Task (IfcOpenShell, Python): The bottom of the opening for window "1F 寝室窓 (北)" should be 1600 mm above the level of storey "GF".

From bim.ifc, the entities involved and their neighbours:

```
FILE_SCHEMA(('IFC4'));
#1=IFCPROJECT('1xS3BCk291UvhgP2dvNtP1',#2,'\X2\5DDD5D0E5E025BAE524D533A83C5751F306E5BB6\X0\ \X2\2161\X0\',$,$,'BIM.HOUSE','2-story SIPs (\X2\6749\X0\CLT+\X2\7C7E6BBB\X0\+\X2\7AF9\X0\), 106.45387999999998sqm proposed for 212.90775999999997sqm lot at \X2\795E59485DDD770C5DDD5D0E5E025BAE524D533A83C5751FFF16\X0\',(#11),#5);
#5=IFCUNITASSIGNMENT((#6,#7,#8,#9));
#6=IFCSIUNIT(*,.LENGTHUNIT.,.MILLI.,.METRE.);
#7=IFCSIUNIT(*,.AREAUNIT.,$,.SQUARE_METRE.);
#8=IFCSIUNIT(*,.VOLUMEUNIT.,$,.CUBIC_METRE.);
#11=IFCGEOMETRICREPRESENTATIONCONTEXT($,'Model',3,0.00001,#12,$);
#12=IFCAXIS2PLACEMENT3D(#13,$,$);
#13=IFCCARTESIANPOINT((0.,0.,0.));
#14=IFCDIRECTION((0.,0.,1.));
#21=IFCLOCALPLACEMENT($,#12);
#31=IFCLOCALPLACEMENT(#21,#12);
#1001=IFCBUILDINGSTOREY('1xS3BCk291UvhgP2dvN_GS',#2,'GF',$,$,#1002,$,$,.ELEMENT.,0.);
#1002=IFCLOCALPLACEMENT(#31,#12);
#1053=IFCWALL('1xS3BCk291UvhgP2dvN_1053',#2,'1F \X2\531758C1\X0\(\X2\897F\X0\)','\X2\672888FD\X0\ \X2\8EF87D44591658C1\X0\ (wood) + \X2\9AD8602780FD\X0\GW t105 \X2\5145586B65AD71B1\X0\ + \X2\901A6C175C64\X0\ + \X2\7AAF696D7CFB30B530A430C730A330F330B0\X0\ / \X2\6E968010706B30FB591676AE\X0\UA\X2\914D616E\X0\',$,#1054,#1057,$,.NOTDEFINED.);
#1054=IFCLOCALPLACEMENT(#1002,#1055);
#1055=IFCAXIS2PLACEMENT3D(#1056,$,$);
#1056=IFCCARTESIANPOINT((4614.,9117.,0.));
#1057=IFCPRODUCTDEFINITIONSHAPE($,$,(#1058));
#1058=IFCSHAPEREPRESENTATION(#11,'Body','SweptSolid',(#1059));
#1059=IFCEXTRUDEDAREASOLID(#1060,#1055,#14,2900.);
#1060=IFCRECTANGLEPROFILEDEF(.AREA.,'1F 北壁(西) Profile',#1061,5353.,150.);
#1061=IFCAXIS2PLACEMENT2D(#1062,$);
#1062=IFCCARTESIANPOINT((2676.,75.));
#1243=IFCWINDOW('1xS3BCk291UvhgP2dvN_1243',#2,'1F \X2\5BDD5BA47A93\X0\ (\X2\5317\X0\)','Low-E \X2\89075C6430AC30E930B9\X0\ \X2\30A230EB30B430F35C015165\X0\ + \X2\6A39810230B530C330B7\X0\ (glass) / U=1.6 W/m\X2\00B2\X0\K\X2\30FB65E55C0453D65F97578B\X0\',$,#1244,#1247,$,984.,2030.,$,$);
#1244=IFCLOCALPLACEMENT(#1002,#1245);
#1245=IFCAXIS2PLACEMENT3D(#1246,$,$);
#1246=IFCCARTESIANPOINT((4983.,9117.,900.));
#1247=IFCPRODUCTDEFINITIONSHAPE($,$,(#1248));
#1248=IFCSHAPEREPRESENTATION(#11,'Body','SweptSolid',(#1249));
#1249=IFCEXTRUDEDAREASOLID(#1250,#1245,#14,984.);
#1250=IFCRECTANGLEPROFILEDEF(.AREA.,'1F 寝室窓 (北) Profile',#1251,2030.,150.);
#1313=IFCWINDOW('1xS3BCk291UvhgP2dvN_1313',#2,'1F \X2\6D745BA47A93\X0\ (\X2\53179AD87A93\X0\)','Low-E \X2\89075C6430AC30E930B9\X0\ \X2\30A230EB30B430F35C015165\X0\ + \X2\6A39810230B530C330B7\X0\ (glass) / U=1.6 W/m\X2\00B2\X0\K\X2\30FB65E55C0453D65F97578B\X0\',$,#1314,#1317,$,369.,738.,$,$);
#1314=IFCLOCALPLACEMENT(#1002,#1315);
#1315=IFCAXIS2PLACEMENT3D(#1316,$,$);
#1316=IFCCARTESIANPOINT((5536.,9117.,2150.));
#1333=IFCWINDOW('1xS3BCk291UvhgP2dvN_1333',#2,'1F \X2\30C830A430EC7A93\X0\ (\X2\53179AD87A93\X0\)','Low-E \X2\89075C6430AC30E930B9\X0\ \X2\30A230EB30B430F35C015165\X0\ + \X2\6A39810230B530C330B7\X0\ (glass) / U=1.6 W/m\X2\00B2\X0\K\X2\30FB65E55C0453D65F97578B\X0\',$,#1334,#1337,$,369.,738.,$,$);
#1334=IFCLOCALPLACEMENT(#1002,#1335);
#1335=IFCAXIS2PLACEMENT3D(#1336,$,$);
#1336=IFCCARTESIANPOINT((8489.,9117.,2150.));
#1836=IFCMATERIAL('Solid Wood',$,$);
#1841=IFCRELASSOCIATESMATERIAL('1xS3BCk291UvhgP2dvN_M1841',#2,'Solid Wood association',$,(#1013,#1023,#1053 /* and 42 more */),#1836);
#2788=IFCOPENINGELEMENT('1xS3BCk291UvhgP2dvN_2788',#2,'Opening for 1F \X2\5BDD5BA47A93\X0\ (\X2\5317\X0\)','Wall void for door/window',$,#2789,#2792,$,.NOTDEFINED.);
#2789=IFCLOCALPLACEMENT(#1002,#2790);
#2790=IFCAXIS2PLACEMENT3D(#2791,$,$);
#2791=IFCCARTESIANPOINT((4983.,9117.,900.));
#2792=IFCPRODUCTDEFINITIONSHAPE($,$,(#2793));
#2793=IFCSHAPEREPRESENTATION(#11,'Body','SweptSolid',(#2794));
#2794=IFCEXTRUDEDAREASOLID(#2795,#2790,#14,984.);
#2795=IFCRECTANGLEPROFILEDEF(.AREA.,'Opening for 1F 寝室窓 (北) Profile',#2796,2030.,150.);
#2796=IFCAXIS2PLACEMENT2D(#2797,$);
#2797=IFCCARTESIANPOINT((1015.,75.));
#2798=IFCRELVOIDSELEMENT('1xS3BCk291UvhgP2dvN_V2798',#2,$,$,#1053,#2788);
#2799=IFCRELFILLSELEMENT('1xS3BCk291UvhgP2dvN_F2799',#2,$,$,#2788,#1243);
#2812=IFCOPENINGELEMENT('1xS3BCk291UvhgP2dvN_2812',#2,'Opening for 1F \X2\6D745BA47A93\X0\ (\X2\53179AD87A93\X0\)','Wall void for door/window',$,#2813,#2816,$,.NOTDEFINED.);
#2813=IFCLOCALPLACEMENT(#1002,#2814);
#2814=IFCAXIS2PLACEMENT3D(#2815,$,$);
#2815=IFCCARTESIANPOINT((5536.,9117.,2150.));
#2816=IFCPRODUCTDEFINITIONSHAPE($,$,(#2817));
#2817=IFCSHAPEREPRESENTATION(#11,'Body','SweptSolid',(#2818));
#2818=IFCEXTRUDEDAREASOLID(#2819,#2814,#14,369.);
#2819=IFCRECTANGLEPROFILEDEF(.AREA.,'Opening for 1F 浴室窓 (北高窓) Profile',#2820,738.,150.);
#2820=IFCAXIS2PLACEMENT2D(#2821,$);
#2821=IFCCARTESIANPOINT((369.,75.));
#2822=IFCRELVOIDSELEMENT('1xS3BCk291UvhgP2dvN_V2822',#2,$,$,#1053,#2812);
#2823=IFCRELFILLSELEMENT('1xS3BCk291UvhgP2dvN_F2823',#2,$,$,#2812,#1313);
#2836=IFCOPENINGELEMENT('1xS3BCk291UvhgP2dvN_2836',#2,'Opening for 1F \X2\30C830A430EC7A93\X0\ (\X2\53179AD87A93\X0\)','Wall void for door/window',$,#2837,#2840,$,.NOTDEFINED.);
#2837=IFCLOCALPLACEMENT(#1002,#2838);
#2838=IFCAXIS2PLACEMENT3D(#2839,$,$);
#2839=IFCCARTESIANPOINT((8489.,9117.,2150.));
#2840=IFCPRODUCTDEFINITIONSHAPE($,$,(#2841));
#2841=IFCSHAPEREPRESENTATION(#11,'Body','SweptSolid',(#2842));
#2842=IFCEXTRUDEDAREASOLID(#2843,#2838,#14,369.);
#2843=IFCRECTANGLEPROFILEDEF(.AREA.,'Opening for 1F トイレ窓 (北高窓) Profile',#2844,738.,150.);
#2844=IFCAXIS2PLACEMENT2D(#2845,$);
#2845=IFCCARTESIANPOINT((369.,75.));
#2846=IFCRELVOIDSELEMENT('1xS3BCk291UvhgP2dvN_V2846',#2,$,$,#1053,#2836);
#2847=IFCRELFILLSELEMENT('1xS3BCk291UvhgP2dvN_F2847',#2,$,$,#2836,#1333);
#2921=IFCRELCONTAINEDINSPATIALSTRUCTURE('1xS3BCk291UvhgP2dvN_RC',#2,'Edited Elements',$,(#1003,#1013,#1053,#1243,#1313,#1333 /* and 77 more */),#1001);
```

```python
import numpy as np
import ifcopenshell
import ifcopenshell.api.geometry
import ifcopenshell.geom
import ifcopenshell.util.element
import ifcopenshell.util.placement
import ifcopenshell.util.shape
import ifcopenshell.util.unit

model = ifcopenshell.open("bim.ifc")
unit_scale = ifcopenshell.util.unit.calculate_unit_scale(model)

window = model.by_guid("1xS3BCk291UvhgP2dvN_1243")
opening = window.FillsVoids[0].RelatingOpeningElement
storey = ifcopenshell.util.element.get_container(window, ifc_class="IfcBuildingStorey")
level = ifcopenshell.util.placement.get_local_placement(storey.ObjectPlacement)[2, 3]

# The opening's origin need not be at the sill, so measure its lowest point.
shape = ifcopenshell.geom.create_shape(ifcopenshell.geom.settings(), opening)
bottom = ifcopenshell.util.shape.get_shape_bottom_elevation(shape, shape.geometry) / unit_scale
dz = level + 1600.0 - bottom

shift = np.array([0.0, 0.0, dz])
# The window is not placed relative to its opening, so move both.
for product in (opening, window):
    matrix = ifcopenshell.util.placement.get_local_placement(product.ObjectPlacement)
    matrix[:3, 3] += shift
    ifcopenshell.api.geometry.edit_object_placement(model, product=product, matrix=matrix, is_si=False)

print(f"moved by {dz * unit_scale:+.3f} m")

model.write("bim_updated.ifc")
```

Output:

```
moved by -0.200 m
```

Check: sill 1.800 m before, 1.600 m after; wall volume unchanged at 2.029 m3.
